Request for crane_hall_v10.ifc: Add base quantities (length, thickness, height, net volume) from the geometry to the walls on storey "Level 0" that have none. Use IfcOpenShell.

First a look at what the model holds.

```python
import ifcopenshell
import ifcopenshell.util.element
import ifcopenshell.util.unit

model = ifcopenshell.open("crane_hall_v10.ifc")
print(model.schema)
for unit_type in ("LENGTHUNIT", "AREAUNIT", "VOLUMEUNIT"):
    print(unit_type, ifcopenshell.util.unit.calculate_unit_scale(model, unit_type))
storey = next(s for s in model.by_type("IfcBuildingStorey") if s.Name == "Level 0")
walls = [e for e in ifcopenshell.util.element.get_decomposition(storey) if e.is_a("IfcWall")]
for e in sorted(walls, key=lambda e: e.id()):
    print(e.id(), e.is_a(), e.Name, list(ifcopenshell.util.element.get_psets(e, qtos_only=True)), sep=" | ")
```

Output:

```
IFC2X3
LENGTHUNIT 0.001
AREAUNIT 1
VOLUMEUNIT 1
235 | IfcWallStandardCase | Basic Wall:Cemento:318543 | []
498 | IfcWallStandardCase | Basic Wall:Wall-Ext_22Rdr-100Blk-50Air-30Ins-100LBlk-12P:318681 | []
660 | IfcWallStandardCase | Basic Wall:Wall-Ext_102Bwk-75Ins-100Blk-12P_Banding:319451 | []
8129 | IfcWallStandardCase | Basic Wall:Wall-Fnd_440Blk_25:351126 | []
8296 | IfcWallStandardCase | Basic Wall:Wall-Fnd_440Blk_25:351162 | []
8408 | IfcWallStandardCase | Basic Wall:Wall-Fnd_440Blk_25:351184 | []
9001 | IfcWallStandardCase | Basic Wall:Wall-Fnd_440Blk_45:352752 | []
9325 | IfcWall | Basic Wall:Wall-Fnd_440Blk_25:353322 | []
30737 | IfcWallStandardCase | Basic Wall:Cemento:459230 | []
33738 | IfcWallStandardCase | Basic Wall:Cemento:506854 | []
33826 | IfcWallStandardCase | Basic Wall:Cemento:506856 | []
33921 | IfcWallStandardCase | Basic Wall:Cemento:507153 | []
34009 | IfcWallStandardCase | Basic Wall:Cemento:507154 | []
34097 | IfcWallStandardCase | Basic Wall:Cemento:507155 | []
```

```python
import ifcopenshell
import ifcopenshell.api.pset
import ifcopenshell.geom
import ifcopenshell.util.element
import ifcopenshell.util.shape
import ifcopenshell.util.unit

model = ifcopenshell.open("crane_hall_v10.ifc")
unit_scale = ifcopenshell.util.unit.calculate_unit_scale(model)
volume_scale = ifcopenshell.util.unit.calculate_unit_scale(model, "VOLUMEUNIT")
settings = ifcopenshell.geom.settings()

storey = next(s for s in model.by_type("IfcBuildingStorey") if s.Name == "Level 0")
walls = [e for e in ifcopenshell.util.element.get_decomposition(storey) if e.is_a("IfcWall")]

for e in sorted(walls, key=lambda e: e.id()):
    if ifcopenshell.util.element.get_psets(e, qtos_only=True, should_inherit=False):
        continue
    # Geometry comes back in metres, in the element's own axes.
    shape = ifcopenshell.geom.create_shape(settings, e)
    values = {
        "Length": ifcopenshell.util.shape.get_x(shape.geometry) / unit_scale,
        "Width": ifcopenshell.util.shape.get_y(shape.geometry) / unit_scale,
        "Height": ifcopenshell.util.shape.get_z(shape.geometry) / unit_scale,
        "NetVolume": ifcopenshell.util.shape.get_volume(shape.geometry) / volume_scale,
    }
    qto = ifcopenshell.api.pset.add_qto(model, product=e, name="BaseQuantities")
    ifcopenshell.api.pset.edit_qto(model, qto=qto, properties=values)
    print(e.id(), {k: round(v, 3) for k, v in values.items()})

model.write("crane_hall_v10_edited.ifc")
```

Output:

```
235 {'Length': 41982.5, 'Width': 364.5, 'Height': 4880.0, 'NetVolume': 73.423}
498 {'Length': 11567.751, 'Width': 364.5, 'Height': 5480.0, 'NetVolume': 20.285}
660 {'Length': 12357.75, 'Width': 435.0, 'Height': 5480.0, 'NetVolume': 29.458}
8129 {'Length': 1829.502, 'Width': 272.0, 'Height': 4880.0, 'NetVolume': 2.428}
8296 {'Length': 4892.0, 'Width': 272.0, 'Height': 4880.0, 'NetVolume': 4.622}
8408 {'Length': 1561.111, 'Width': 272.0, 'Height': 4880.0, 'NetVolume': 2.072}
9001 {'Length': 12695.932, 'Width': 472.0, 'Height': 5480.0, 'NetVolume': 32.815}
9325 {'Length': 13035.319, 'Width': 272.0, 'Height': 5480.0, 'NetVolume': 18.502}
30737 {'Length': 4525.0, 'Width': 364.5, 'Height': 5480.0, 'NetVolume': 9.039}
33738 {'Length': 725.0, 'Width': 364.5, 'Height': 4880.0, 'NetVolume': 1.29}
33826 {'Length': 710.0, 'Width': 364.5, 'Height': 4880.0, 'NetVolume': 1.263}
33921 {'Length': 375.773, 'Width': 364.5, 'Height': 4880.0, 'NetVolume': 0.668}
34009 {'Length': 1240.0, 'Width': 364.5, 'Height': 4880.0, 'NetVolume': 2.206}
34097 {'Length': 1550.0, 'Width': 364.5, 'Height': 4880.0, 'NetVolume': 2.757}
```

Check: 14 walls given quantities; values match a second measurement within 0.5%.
